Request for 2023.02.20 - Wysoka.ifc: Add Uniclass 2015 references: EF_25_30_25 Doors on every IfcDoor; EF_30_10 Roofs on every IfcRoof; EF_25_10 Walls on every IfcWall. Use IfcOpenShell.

First a look at what the model holds.

```python
import ifcopenshell

model = ifcopenshell.open("2023.02.20 - Wysoka.ifc")
print(model.schema)
print("classifications:", [c.Name for c in model.by_type("IfcClassification")])
for ifc_class in ("IfcDoor", "IfcRoof", "IfcStair", "IfcWall", "IfcWindow"):
    print(ifc_class, len(model.by_type(ifc_class)))
```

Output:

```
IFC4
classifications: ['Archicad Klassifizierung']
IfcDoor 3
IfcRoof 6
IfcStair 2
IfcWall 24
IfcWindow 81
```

```python
import ifcopenshell
import ifcopenshell.api.classification

model = ifcopenshell.open("2023.02.20 - Wysoka.ifc")

system = ifcopenshell.api.classification.add_classification(model, classification="Uniclass 2015")

codes = {
    "IfcDoor": ("EF_25_30_25", "Doors"),
    "IfcRoof": ("EF_30_10", "Roofs"),
    "IfcWall": ("EF_25_10", "Walls"),
}
for ifc_class, (code, name) in codes.items():
    products = model.by_type(ifc_class)
    ifcopenshell.api.classification.add_reference(
        model, products=products, classification=system, identification=code, name=name
    )
    print(code, len(products))

model.write("2023.02.20 - Wysoka_updated.ifc")
```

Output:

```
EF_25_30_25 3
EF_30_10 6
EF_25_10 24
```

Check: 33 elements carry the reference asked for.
